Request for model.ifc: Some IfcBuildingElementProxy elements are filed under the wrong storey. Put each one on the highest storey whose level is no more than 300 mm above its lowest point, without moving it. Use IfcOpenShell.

First a look at what the model holds.

```python
import ifcopenshell
import ifcopenshell.util.element
import ifcopenshell.util.placement

model = ifcopenshell.open("model.ifc")
print(model.schema)
for storey in model.by_type("IfcBuildingStorey"):
    level = ifcopenshell.util.placement.get_storey_elevation(storey)
    count = sum(e.is_a("IfcBuildingElementProxy") for e in ifcopenshell.util.element.get_contained(storey))
    print(storey.id(), storey.Name, round(level, 3), count, sep=" | ")
```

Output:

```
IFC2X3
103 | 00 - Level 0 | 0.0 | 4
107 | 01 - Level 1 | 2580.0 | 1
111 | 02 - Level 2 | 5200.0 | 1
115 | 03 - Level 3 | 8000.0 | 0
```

```python
import ifcopenshell
import ifcopenshell.api.spatial
import ifcopenshell.geom
import ifcopenshell.util.element
import ifcopenshell.util.placement
import ifcopenshell.util.shape
import ifcopenshell.util.unit

model = ifcopenshell.open("model.ifc")
unit_scale = ifcopenshell.util.unit.calculate_unit_scale(model)
settings = ifcopenshell.geom.settings()

levels = sorted(
    ((ifcopenshell.util.placement.get_storey_elevation(s) * unit_scale, s) for s in model.by_type("IfcBuildingStorey")),
    key=lambda pair: pair[0],
)

for e in model.by_type("IfcBuildingElementProxy"):
    current = e.ContainedInStructure[0].RelatingStructure if e.ContainedInStructure else None
    if current is None or not current.is_a("IfcBuildingStorey"):
        continue
    shape = ifcopenshell.geom.create_shape(settings, e)
    bottom = ifcopenshell.util.shape.get_shape_bottom_elevation(shape, shape.geometry)
    below = [s for level, s in levels if level <= bottom + 0.3]
    storey = below[-1] if below else levels[0][1]
    if storey != current:
        # assign_container keeps the world position.
        ifcopenshell.api.spatial.assign_container(model, products=[e], relating_structure=storey)
        print(e.id(), current.Name, "->", storey.Name)

model.write("model_updated.ifc")
```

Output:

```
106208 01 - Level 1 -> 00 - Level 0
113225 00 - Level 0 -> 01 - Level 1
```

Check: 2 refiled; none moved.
